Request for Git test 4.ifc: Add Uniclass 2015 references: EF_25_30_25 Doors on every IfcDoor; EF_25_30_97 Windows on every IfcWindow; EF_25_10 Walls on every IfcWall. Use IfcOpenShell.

First a look at what the model holds.

```python
import ifcopenshell

model = ifcopenshell.open("Git test 4.ifc")
print(model.schema)
print("classifications:", [c.Name for c in model.by_type("IfcClassification")])
for ifc_class in ("IfcDoor", "IfcRoof", "IfcStair", "IfcWall", "IfcWindow"):
    print(ifc_class, len(model.by_type(ifc_class)))
```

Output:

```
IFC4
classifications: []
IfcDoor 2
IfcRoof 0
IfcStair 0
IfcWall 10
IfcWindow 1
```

```python
import ifcopenshell
import ifcopenshell.api.classification

model = ifcopenshell.open("Git test 4.ifc")

system = ifcopenshell.api.classification.add_classification(model, classification="Uniclass 2015")

codes = {
    "IfcDoor": ("EF_25_30_25", "Doors"),
    "IfcWindow": ("EF_25_30_97", "Windows"),
    "IfcWall": ("EF_25_10", "Walls"),
}
for ifc_class, (code, name) in codes.items():
    products = model.by_type(ifc_class)
    ifcopenshell.api.classification.add_reference(
        model, products=products, classification=system, identification=code, name=name
    )
    print(code, len(products))

model.write("Git test 4_rev.ifc")
```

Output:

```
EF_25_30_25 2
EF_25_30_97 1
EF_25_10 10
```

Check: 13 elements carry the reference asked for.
